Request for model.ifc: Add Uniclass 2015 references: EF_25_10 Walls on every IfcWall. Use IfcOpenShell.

First a look at what the model holds.

```python
import ifcopenshell

model = ifcopenshell.open("model.ifc")
print(model.schema)
print("classifications:", [c.Name for c in model.by_type("IfcClassification")])
for ifc_class in ("IfcDoor", "IfcRoof", "IfcStair", "IfcWall", "IfcWindow"):
    print(ifc_class, len(model.by_type(ifc_class)))
```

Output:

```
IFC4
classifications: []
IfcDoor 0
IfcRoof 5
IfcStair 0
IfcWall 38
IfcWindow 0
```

```python
import ifcopenshell
import ifcopenshell.api.classification

model = ifcopenshell.open("model.ifc")

system = ifcopenshell.api.classification.add_classification(model, classification="Uniclass 2015")

codes = {
    "IfcWall": ("EF_25_10", "Walls"),
}
for ifc_class, (code, name) in codes.items():
    products = model.by_type(ifc_class)
    ifcopenshell.api.classification.add_reference(
        model, products=products, classification=system, identification=code, name=name
    )
    print(code, len(products))

model.write("model_edited.ifc")
```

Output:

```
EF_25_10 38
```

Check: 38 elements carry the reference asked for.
